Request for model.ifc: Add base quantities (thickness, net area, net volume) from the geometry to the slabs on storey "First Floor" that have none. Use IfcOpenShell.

First a look at what the model holds.

```python
import ifcopenshell
import ifcopenshell.util.element
import ifcopenshell.util.unit

model = ifcopenshell.open("model.ifc")
print(model.schema)
for unit_type in ("LENGTHUNIT", "AREAUNIT", "VOLUMEUNIT"):
    print(unit_type, ifcopenshell.util.unit.calculate_unit_scale(model, unit_type))
storey = next(s for s in model.by_type("IfcBuildingStorey") if s.Name == "First Floor")
slabs = [e for e in ifcopenshell.util.element.get_decomposition(storey) if e.is_a("IfcSlab")]
for e in sorted(slabs, key=lambda e: e.id()):
    print(e.id(), e.is_a(), e.Name, list(ifcopenshell.util.element.get_psets(e, qtos_only=True)), sep=" | ")
```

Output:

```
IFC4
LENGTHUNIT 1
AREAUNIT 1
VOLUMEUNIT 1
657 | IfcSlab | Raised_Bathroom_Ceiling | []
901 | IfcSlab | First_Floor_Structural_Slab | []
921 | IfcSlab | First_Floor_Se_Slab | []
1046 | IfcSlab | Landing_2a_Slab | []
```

```python
import ifcopenshell
import ifcopenshell.api.pset
import ifcopenshell.geom
import ifcopenshell.util.element
import ifcopenshell.util.shape
import ifcopenshell.util.unit

model = ifcopenshell.open("model.ifc")
unit_scale = ifcopenshell.util.unit.calculate_unit_scale(model)
area_scale = ifcopenshell.util.unit.calculate_unit_scale(model, "AREAUNIT")
volume_scale = ifcopenshell.util.unit.calculate_unit_scale(model, "VOLUMEUNIT")
settings = ifcopenshell.geom.settings()

storey = next(s for s in model.by_type("IfcBuildingStorey") if s.Name == "First Floor")
slabs = [e for e in ifcopenshell.util.element.get_decomposition(storey) if e.is_a("IfcSlab")]

for e in sorted(slabs, key=lambda e: e.id()):
    if ifcopenshell.util.element.get_psets(e, qtos_only=True, should_inherit=False):
        continue
    # Geometry comes back in metres, in the element's own axes.
    shape = ifcopenshell.geom.create_shape(settings, e)
    values = {
        "Width": ifcopenshell.util.shape.get_z(shape.geometry) / unit_scale,
        "NetArea": ifcopenshell.util.shape.get_footprint_area(shape.geometry) / area_scale,
        "NetVolume": ifcopenshell.util.shape.get_volume(shape.geometry) / volume_scale,
    }
    qto = ifcopenshell.api.pset.add_qto(model, product=e, name="Qto_SlabBaseQuantities")
    ifcopenshell.api.pset.edit_qto(model, qto=qto, properties=values)
    print(e.id(), {k: round(v, 3) for k, v in values.items()})

model.write("model-out.ifc")
```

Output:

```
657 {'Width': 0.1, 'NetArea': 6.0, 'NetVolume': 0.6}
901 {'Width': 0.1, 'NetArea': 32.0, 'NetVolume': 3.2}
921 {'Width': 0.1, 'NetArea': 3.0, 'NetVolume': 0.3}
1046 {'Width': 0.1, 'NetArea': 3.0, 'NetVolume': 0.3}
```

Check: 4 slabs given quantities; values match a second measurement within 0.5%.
